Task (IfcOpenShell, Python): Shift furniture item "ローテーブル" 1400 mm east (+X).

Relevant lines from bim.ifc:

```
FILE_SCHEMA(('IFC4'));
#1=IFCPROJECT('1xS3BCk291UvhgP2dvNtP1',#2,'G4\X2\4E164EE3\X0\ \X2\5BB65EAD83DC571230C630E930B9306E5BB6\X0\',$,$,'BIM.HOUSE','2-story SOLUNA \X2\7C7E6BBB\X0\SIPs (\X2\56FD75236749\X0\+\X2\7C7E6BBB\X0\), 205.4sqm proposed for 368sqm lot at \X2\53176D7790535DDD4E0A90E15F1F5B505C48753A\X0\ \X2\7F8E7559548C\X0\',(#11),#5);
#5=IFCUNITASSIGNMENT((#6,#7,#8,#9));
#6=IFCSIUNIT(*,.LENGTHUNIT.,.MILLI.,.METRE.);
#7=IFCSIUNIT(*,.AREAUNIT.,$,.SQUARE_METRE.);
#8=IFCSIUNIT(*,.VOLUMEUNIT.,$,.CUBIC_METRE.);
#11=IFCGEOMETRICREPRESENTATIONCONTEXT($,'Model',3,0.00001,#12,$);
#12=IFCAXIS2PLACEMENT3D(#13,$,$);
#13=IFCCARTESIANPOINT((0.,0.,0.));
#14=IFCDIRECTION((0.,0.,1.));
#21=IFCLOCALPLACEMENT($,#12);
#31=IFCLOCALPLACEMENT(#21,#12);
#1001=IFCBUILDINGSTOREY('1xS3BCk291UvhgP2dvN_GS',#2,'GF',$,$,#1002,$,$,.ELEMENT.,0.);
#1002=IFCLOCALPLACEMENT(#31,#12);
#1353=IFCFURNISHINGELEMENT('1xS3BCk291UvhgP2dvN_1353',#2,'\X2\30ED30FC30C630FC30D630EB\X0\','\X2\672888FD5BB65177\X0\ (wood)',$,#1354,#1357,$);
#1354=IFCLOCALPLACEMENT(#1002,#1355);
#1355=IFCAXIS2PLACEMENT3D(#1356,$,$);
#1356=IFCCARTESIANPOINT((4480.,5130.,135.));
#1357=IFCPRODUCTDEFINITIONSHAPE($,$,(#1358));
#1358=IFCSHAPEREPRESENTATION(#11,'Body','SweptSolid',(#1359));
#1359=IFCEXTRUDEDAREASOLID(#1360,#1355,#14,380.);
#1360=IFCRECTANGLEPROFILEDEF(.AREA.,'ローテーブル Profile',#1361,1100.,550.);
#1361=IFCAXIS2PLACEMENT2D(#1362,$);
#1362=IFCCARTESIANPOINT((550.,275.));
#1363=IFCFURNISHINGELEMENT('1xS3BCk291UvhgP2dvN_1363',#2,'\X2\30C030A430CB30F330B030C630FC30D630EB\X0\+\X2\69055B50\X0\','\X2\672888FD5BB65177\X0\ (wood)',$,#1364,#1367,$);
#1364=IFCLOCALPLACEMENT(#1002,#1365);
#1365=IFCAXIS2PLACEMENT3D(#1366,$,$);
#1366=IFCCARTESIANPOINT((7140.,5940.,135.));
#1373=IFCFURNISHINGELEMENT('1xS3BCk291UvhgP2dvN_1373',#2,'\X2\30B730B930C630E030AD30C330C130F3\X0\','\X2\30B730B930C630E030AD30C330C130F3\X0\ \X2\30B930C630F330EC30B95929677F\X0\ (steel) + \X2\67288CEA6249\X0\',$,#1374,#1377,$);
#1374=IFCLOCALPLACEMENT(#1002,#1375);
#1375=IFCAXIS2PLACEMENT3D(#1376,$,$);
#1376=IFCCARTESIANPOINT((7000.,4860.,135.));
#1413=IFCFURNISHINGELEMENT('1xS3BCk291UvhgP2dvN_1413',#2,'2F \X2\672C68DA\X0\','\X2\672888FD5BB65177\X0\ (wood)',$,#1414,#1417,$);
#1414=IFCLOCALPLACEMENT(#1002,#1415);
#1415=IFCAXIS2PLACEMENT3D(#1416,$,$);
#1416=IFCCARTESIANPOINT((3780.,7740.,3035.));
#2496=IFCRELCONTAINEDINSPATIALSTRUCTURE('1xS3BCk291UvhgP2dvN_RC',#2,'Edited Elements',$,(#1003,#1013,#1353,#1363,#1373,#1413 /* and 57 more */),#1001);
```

```python
import ifcopenshell
import ifcopenshell.api.geometry
import ifcopenshell.util.placement
import ifcopenshell.util.unit

model = ifcopenshell.open("bim.ifc")
unit_scale = ifcopenshell.util.unit.calculate_unit_scale(model)

item = model.by_guid("1xS3BCk291UvhgP2dvN_1353")
matrix = ifcopenshell.util.placement.get_local_placement(item.ObjectPlacement)
matrix[0, 3] += 1.4 / unit_scale
ifcopenshell.api.geometry.edit_object_placement(model, product=item, matrix=matrix, is_si=False)

print(ifcopenshell.util.placement.get_local_placement(item.ObjectPlacement).round(3) + 0.0)

model.write("bim_edited.ifc")
```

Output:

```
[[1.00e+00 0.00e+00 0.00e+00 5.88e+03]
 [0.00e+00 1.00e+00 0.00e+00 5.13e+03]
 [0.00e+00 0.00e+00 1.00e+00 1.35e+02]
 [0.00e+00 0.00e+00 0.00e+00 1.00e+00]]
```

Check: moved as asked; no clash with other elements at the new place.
